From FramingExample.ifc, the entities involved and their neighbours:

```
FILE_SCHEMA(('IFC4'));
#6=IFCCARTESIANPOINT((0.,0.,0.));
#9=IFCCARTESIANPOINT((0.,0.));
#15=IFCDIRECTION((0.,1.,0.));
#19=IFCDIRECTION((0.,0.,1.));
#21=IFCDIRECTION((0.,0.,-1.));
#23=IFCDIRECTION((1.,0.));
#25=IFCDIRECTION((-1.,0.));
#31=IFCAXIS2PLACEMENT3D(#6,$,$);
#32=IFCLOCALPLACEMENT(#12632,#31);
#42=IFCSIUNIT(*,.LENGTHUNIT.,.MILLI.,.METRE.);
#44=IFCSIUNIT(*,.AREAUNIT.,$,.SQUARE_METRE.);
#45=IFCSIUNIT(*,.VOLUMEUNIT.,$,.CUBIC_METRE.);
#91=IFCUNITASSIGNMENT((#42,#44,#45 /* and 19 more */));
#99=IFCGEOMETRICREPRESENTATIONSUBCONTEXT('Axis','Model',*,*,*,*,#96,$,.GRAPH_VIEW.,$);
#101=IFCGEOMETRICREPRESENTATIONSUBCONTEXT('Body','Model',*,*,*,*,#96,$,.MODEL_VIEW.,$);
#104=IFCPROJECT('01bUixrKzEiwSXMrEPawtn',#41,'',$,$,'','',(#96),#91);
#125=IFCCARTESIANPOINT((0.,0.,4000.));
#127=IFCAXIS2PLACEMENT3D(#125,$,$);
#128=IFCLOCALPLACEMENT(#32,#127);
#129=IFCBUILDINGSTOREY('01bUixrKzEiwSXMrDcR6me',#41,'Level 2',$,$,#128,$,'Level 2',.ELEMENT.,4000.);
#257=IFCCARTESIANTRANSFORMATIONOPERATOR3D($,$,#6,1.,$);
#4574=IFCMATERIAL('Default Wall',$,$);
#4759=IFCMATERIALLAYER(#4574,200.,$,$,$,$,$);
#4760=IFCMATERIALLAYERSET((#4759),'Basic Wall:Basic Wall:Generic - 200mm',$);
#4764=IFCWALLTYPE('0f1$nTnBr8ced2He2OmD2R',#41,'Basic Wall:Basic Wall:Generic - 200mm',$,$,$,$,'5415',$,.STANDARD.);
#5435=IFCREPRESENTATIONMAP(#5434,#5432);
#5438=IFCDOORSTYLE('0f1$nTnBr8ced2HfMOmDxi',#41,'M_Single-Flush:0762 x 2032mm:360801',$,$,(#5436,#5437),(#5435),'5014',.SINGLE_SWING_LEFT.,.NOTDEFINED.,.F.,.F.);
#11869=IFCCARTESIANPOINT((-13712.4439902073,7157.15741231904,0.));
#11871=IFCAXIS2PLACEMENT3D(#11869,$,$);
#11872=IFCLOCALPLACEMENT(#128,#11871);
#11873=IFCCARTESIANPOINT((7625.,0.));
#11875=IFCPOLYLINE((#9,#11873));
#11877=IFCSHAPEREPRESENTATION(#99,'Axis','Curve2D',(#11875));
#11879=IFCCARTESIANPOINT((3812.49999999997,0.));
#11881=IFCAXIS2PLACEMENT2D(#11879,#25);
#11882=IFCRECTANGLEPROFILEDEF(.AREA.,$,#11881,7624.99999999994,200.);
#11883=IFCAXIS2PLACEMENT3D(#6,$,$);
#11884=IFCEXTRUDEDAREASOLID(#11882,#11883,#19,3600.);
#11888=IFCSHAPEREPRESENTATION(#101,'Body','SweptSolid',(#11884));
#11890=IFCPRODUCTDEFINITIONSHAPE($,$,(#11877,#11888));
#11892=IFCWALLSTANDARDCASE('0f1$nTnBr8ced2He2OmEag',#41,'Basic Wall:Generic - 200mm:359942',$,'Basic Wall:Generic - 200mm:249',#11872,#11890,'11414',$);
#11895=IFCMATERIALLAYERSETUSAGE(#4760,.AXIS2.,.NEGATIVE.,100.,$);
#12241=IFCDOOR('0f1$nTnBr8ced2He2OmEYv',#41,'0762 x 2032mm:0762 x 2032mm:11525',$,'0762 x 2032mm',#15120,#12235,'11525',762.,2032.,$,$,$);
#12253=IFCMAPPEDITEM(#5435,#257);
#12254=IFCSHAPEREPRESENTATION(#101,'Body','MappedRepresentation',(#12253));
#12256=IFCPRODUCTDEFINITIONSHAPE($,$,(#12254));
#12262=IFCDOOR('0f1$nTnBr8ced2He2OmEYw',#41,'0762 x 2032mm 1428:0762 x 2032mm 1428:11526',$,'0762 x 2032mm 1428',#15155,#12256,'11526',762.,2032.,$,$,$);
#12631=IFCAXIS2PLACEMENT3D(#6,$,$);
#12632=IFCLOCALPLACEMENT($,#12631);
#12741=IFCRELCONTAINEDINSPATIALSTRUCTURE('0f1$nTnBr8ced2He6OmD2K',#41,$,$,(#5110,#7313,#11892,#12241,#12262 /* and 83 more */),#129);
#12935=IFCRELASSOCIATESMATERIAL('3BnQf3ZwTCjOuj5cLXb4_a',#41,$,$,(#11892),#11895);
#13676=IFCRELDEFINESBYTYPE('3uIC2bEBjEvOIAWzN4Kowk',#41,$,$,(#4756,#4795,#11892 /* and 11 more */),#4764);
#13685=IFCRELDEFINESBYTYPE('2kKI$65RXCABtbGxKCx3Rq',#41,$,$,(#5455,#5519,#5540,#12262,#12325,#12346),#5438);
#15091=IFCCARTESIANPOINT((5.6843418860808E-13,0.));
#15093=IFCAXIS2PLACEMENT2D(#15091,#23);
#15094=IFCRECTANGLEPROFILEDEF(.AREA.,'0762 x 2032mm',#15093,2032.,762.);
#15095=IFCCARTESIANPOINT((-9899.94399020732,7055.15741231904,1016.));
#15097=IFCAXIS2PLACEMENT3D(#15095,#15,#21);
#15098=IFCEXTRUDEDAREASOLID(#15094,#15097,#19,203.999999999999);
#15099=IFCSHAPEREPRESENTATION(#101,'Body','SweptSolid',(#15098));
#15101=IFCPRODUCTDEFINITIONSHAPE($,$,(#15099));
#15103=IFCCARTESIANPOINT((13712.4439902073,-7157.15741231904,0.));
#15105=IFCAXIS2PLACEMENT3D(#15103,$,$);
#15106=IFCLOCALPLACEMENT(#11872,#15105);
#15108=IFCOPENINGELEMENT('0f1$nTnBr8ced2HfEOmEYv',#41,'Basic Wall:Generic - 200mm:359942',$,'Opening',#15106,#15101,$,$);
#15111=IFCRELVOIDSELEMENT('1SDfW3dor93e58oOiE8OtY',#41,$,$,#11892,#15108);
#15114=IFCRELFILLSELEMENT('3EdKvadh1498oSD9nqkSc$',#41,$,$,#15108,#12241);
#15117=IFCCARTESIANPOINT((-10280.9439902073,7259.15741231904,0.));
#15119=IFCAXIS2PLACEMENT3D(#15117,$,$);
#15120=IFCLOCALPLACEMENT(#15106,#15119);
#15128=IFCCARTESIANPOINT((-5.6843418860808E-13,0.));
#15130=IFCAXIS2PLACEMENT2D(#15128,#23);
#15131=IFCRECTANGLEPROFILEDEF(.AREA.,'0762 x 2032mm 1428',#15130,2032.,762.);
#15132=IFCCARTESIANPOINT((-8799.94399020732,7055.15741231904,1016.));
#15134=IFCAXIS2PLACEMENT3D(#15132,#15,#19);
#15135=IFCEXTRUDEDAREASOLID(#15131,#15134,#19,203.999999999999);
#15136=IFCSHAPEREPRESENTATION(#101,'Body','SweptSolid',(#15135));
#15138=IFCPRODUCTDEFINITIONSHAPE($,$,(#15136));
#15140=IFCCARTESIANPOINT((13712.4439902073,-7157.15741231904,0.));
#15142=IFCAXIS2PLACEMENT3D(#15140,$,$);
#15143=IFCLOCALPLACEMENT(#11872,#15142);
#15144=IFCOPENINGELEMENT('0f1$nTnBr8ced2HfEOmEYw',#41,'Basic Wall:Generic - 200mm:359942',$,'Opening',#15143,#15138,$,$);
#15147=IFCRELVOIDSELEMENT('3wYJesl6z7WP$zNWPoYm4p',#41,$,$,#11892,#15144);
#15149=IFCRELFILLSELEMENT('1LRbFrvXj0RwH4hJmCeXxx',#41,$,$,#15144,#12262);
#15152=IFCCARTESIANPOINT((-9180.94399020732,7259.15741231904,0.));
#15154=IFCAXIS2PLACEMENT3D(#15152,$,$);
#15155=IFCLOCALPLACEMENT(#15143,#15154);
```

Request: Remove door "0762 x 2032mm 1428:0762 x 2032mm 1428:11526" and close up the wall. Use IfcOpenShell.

```python
import ifcopenshell
import ifcopenshell.api.feature
import ifcopenshell.api.root
import ifcopenshell.geom
import ifcopenshell.util.shape

model = ifcopenshell.open("FramingExample.ifc")
settings = ifcopenshell.geom.settings()


def volume(element):
    """Net volume in cubic metres, openings subtracted."""
    shape = ifcopenshell.geom.create_shape(settings, element)
    return ifcopenshell.util.shape.get_volume(shape.geometry)


door = model.by_guid("0f1$nTnBr8ced2He2OmEYw")
opening = door.FillsVoids[0].RelatingOpeningElement
wall = opening.VoidsElements[0].RelatingBuildingElement
before = volume(wall)

ifcopenshell.api.root.remove_product(model, product=door)
ifcopenshell.api.feature.remove_feature(model, feature=opening)

after = volume(wall)

print(f"wall volume {before:.3f} -> {after:.3f} m3")

model.write("FramingExample-out.ifc")
```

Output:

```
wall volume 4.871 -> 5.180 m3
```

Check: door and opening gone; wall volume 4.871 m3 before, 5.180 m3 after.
